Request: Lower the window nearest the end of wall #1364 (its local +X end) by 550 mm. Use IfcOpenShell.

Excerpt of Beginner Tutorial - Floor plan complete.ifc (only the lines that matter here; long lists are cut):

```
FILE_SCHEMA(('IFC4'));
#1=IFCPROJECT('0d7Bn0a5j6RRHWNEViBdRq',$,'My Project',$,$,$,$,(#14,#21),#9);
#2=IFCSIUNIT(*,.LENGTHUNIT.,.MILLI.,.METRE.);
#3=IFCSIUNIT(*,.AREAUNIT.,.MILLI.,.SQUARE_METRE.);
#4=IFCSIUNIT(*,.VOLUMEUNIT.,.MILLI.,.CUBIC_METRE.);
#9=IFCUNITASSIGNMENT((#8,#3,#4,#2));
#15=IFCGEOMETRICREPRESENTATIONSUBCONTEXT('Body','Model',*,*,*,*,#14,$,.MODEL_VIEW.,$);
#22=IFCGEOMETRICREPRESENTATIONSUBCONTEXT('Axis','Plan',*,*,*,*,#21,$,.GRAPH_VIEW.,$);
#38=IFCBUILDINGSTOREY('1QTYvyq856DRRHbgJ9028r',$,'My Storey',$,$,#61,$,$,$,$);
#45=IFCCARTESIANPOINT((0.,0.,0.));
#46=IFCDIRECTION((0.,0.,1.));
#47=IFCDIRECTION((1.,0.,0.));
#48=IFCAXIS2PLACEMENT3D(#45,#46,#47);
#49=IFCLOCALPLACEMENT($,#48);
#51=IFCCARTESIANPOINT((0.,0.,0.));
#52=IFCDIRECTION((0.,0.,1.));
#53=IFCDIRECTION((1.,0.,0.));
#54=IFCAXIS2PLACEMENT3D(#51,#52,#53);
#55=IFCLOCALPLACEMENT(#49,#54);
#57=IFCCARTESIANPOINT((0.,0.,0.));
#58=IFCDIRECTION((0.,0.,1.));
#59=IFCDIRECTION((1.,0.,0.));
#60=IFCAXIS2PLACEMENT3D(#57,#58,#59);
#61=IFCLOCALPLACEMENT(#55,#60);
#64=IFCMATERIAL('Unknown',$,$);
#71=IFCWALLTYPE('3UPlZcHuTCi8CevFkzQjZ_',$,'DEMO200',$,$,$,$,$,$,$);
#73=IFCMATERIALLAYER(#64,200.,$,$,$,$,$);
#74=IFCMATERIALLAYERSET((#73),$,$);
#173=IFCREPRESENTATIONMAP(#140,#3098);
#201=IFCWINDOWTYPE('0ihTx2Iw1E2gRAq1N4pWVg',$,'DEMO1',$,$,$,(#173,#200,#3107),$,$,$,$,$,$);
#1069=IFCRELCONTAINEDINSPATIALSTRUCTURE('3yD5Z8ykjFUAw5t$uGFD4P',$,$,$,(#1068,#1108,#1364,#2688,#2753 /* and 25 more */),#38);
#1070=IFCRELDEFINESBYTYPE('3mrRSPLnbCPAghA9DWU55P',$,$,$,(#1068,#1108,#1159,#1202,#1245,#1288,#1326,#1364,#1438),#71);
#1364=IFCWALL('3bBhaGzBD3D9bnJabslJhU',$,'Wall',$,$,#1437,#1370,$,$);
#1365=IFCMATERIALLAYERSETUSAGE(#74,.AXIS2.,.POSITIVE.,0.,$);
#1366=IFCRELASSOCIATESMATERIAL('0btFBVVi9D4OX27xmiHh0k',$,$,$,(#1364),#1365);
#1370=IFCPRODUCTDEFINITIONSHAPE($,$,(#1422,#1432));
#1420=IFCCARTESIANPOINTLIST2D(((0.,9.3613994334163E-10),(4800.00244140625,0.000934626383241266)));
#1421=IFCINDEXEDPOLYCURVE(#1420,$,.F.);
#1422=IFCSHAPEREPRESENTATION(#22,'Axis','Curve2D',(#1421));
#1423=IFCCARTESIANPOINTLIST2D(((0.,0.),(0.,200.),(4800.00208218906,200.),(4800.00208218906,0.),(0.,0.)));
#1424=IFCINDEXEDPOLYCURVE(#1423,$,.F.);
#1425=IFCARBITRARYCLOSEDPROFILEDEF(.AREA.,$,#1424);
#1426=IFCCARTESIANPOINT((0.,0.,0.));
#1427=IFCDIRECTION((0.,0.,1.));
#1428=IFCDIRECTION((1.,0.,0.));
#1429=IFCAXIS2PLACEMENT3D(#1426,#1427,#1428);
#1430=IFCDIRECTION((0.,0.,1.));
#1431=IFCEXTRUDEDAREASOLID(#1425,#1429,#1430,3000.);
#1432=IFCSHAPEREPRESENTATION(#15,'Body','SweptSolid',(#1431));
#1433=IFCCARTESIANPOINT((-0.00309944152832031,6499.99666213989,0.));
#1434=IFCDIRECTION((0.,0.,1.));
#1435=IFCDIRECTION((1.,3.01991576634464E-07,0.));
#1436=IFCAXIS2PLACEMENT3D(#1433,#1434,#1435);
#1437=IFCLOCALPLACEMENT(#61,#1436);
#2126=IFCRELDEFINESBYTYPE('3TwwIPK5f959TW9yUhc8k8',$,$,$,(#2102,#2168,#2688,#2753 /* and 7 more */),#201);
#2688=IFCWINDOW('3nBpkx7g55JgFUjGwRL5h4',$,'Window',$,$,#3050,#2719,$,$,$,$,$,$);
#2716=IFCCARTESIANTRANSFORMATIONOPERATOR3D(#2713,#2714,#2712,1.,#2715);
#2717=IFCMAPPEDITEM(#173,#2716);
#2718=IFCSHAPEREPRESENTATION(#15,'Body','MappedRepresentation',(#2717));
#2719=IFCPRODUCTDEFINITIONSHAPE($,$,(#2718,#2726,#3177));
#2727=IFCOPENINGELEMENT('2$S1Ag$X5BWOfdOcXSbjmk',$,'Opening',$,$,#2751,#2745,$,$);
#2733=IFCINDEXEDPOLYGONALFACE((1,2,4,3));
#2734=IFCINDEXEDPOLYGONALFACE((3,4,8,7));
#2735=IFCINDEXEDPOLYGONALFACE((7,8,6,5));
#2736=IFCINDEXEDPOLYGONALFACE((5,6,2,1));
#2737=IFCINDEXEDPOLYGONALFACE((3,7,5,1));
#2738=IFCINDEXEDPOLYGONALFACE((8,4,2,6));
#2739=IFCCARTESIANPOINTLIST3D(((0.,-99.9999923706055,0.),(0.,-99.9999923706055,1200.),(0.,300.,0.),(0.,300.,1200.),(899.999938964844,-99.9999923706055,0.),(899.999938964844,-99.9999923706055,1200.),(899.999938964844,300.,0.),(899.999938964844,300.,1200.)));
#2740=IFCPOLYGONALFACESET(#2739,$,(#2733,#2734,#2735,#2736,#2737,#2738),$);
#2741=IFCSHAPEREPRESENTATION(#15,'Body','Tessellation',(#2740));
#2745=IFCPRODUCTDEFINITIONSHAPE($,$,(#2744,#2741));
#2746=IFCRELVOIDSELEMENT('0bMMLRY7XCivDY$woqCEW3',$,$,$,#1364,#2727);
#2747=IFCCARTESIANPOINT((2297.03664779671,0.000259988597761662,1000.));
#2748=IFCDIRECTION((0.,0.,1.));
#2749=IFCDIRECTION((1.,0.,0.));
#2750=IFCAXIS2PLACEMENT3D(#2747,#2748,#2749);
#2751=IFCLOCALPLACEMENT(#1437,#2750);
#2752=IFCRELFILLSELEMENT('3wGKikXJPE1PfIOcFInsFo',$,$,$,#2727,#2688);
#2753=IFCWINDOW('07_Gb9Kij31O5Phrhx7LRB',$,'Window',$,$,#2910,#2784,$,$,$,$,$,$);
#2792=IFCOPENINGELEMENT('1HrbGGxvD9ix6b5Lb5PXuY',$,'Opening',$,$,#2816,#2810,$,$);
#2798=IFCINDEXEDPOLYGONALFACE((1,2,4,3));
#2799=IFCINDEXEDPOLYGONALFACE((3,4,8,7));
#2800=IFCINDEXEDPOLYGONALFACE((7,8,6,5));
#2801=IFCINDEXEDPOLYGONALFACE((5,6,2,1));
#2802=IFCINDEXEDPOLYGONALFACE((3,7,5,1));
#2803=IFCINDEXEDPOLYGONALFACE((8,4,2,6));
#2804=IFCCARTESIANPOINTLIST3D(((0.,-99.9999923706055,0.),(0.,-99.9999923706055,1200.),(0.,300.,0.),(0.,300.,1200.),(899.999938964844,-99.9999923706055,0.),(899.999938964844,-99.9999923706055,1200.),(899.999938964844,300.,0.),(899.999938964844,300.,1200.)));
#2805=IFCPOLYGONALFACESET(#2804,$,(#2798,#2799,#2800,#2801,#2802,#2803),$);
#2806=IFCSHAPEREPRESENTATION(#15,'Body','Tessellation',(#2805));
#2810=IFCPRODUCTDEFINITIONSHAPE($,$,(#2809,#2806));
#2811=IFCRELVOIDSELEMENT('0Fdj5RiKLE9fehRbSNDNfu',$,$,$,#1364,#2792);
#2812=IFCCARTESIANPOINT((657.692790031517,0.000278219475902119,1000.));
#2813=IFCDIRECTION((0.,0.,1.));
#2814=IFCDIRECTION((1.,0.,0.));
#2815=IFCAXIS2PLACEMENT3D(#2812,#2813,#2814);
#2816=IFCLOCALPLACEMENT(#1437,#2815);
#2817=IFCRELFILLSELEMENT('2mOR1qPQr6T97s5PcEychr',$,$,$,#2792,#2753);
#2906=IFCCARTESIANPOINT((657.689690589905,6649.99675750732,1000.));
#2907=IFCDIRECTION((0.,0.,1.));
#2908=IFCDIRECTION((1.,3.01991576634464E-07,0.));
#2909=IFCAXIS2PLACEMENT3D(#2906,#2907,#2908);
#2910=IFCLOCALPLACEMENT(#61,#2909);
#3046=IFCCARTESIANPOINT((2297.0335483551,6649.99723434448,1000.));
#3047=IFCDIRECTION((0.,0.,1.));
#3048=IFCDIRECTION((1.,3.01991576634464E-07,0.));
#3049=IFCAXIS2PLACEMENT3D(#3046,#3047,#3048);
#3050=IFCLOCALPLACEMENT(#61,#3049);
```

```python
import numpy as np
import ifcopenshell
import ifcopenshell.api.geometry
import ifcopenshell.util.placement
import ifcopenshell.util.unit

model = ifcopenshell.open("Beginner Tutorial - Floor plan complete.ifc")
unit_scale = ifcopenshell.util.unit.calculate_unit_scale(model)

window = model.by_guid("3nBpkx7g55JgFUjGwRL5h4")
opening = window.FillsVoids[0].RelatingOpeningElement
dz = -0.55 / unit_scale

shift = np.array([0.0, 0.0, dz])
# The window is not placed relative to its opening, so move both.
for product in (opening, window):
    matrix = ifcopenshell.util.placement.get_local_placement(product.ObjectPlacement)
    matrix[:3, 3] += shift
    ifcopenshell.api.geometry.edit_object_placement(model, product=product, matrix=matrix, is_si=False)

print(f"moved by {dz * unit_scale:+.3f} m")

model.write("Beginner Tutorial - Floor plan complete_updated.ifc")
```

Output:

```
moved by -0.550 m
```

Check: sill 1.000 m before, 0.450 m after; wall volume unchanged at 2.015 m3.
